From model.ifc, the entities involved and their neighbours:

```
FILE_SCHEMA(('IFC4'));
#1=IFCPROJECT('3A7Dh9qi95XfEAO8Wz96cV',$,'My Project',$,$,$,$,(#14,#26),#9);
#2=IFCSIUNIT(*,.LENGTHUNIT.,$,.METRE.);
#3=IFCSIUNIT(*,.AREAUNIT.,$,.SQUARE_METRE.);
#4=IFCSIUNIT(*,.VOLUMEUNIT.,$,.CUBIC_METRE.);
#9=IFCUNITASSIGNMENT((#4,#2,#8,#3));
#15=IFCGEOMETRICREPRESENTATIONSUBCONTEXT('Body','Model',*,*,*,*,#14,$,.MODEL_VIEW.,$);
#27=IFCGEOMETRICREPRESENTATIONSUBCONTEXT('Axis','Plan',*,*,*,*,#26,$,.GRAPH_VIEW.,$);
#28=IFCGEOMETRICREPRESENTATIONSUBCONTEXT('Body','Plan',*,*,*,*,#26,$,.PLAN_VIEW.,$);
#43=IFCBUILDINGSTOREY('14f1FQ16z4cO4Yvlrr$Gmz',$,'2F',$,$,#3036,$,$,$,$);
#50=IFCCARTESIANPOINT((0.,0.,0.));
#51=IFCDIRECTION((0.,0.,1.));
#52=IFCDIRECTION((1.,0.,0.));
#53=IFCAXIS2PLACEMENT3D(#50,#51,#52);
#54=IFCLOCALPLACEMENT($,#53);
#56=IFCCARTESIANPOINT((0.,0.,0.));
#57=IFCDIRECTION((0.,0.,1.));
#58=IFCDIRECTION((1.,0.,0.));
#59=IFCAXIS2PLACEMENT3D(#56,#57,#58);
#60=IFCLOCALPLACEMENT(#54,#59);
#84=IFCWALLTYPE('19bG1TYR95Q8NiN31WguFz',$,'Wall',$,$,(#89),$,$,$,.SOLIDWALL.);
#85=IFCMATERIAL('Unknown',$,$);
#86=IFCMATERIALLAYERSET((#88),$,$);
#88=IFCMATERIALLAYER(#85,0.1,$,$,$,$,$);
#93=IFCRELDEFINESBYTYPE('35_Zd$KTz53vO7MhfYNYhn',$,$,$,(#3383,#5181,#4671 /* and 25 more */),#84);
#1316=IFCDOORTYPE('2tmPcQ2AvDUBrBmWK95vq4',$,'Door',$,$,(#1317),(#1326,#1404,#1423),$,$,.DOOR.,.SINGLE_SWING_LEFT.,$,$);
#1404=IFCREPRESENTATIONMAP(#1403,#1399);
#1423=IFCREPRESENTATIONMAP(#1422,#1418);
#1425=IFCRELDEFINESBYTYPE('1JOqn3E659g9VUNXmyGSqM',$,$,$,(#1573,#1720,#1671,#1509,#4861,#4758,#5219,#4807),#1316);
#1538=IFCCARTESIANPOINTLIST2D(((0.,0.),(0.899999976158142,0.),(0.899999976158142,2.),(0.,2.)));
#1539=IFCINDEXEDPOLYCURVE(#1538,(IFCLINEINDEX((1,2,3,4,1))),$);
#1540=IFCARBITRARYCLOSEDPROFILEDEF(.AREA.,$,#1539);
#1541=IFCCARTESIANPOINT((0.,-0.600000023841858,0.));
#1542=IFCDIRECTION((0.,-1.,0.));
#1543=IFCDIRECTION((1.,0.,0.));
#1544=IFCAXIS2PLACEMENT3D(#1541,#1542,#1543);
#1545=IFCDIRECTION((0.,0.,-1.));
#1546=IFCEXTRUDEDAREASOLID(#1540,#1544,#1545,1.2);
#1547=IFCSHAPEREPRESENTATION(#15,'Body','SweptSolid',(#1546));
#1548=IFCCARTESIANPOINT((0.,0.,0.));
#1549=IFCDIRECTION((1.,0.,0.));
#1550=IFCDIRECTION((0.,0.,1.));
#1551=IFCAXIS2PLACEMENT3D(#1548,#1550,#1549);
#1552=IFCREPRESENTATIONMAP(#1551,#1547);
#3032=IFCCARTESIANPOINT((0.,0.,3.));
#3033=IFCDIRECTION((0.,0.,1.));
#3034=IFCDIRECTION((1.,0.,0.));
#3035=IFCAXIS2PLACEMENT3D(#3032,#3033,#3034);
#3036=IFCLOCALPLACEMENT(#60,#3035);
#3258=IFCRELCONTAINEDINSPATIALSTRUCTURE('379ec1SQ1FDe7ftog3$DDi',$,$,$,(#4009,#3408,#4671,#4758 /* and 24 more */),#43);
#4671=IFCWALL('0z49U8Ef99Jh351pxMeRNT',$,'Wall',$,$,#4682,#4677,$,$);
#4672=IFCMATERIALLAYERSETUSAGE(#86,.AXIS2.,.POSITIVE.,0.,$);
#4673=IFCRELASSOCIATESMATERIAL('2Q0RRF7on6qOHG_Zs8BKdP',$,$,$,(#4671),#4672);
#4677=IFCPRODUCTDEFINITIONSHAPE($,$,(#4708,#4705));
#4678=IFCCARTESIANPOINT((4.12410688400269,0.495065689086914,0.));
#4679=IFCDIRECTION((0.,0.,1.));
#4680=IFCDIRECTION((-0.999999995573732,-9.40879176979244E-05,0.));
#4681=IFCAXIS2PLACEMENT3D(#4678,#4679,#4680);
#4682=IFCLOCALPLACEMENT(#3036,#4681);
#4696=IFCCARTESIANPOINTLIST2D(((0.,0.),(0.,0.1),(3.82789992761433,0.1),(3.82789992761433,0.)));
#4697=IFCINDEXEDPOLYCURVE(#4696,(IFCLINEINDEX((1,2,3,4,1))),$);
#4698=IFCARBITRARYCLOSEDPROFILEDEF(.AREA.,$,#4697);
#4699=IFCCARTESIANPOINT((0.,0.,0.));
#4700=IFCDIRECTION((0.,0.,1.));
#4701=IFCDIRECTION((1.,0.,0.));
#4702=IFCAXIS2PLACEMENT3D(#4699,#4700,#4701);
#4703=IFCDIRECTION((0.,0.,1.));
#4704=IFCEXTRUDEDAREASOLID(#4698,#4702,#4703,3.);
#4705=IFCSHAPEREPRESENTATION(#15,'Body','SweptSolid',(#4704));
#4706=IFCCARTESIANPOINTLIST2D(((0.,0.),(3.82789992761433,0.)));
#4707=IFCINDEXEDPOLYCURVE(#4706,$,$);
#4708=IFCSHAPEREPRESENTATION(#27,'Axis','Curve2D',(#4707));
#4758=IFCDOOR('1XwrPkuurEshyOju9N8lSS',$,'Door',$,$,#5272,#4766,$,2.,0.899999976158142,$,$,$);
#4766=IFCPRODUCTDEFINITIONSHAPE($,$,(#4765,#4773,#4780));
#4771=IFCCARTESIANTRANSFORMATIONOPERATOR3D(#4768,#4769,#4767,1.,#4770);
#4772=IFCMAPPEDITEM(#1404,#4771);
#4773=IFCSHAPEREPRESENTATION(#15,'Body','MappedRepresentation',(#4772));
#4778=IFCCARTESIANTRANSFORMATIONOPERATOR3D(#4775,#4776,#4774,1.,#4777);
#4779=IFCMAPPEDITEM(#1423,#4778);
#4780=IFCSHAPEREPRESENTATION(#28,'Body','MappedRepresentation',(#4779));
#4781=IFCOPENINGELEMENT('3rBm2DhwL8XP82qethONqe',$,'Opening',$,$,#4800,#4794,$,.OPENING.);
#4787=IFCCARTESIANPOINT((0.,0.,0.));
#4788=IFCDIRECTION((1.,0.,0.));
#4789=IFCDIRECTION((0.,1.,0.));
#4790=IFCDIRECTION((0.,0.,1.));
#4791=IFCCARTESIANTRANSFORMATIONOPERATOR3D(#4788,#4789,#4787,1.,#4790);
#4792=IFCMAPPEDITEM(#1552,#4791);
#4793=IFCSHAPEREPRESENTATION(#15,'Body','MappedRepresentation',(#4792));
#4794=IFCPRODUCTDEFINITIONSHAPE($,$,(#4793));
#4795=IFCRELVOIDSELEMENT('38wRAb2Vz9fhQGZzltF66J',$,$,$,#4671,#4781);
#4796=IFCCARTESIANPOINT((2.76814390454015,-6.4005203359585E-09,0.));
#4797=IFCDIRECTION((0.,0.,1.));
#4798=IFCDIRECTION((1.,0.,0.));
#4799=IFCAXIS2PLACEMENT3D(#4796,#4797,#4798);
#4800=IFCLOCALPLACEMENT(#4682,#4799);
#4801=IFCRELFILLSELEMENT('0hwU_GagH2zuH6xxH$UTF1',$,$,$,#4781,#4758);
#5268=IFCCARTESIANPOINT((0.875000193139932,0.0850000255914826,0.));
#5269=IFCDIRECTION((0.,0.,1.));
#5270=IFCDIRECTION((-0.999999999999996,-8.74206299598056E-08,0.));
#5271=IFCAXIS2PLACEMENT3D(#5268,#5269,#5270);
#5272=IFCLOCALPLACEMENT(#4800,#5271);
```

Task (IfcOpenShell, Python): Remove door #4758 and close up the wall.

```python
import ifcopenshell
import ifcopenshell.api.feature
import ifcopenshell.api.root
import ifcopenshell.geom
import ifcopenshell.util.shape

model = ifcopenshell.open("model.ifc")
settings = ifcopenshell.geom.settings()


def volume(element):
    """Net volume in cubic metres, openings subtracted."""
    shape = ifcopenshell.geom.create_shape(settings, element)
    return ifcopenshell.util.shape.get_volume(shape.geometry)


door = model.by_guid("1XwrPkuurEshyOju9N8lSS")
opening = door.FillsVoids[0].RelatingOpeningElement
wall = opening.VoidsElements[0].RelatingBuildingElement
before = volume(wall)

ifcopenshell.api.root.remove_product(model, product=door)
ifcopenshell.api.feature.remove_feature(model, feature=opening)

after = volume(wall)

print(f"wall volume {before:.3f} -> {after:.3f} m3")

model.write("model_rev.ifc")
```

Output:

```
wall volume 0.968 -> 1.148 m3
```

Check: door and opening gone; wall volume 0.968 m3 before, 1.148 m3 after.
